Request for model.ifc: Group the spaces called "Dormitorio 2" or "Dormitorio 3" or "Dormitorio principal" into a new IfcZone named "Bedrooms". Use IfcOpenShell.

First a look at what the model holds.

```python
import ifcopenshell

model = ifcopenshell.open("model.ifc")
print(model.schema)
seen = {}
for space in model.by_type("IfcSpace"):
    seen[space.LongName] = seen.get(space.LongName, 0) + 1
for name, count in sorted(seen.items(), key=str):
    print(count, "x", name)
print("zones:", [z.Name for z in model.by_type("IfcZone")][:20])
```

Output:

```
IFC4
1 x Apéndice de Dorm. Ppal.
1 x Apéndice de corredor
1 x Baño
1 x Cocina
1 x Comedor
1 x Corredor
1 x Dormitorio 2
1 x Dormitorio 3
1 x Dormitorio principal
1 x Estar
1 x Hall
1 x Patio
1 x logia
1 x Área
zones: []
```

```python
import ifcopenshell
import ifcopenshell.api.group
import ifcopenshell.api.root

model = ifcopenshell.open("model.ifc")

names = {"Dormitorio 2", "Dormitorio 3", "Dormitorio principal"}
spaces = [s for s in model.by_type("IfcSpace") if s.LongName in names]

zone = ifcopenshell.api.root.create_entity(model, ifc_class="IfcZone", name="Bedrooms")
ifcopenshell.api.group.assign_group(model, products=spaces, group=zone)
print(len(spaces), "spaces in", zone.Name)

model.write("model_rev.ifc")
```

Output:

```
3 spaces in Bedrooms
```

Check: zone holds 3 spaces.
